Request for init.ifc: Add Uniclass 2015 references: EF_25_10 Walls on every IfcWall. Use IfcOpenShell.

First a look at what the model holds.

```python
import ifcopenshell

model = ifcopenshell.open("init.ifc")
print(model.schema)
print("classifications:", [c.Name for c in model.by_type("IfcClassification")])
for ifc_class in ("IfcDoor", "IfcRoof", "IfcStair", "IfcWall", "IfcWindow"):
    print(ifc_class, len(model.by_type(ifc_class)))
```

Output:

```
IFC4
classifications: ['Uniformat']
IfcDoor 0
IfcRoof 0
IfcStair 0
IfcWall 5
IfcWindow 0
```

```python
import ifcopenshell
import ifcopenshell.api.classification

model = ifcopenshell.open("init.ifc")

system = ifcopenshell.api.classification.add_classification(model, classification="Uniclass 2015")

codes = {
    "IfcWall": ("EF_25_10", "Walls"),
}
for ifc_class, (code, name) in codes.items():
    products = model.by_type(ifc_class)
    ifcopenshell.api.classification.add_reference(
        model, products=products, classification=system, identification=code, name=name
    )
    print(code, len(products))

model.write("init_rev.ifc")
```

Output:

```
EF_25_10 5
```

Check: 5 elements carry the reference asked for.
